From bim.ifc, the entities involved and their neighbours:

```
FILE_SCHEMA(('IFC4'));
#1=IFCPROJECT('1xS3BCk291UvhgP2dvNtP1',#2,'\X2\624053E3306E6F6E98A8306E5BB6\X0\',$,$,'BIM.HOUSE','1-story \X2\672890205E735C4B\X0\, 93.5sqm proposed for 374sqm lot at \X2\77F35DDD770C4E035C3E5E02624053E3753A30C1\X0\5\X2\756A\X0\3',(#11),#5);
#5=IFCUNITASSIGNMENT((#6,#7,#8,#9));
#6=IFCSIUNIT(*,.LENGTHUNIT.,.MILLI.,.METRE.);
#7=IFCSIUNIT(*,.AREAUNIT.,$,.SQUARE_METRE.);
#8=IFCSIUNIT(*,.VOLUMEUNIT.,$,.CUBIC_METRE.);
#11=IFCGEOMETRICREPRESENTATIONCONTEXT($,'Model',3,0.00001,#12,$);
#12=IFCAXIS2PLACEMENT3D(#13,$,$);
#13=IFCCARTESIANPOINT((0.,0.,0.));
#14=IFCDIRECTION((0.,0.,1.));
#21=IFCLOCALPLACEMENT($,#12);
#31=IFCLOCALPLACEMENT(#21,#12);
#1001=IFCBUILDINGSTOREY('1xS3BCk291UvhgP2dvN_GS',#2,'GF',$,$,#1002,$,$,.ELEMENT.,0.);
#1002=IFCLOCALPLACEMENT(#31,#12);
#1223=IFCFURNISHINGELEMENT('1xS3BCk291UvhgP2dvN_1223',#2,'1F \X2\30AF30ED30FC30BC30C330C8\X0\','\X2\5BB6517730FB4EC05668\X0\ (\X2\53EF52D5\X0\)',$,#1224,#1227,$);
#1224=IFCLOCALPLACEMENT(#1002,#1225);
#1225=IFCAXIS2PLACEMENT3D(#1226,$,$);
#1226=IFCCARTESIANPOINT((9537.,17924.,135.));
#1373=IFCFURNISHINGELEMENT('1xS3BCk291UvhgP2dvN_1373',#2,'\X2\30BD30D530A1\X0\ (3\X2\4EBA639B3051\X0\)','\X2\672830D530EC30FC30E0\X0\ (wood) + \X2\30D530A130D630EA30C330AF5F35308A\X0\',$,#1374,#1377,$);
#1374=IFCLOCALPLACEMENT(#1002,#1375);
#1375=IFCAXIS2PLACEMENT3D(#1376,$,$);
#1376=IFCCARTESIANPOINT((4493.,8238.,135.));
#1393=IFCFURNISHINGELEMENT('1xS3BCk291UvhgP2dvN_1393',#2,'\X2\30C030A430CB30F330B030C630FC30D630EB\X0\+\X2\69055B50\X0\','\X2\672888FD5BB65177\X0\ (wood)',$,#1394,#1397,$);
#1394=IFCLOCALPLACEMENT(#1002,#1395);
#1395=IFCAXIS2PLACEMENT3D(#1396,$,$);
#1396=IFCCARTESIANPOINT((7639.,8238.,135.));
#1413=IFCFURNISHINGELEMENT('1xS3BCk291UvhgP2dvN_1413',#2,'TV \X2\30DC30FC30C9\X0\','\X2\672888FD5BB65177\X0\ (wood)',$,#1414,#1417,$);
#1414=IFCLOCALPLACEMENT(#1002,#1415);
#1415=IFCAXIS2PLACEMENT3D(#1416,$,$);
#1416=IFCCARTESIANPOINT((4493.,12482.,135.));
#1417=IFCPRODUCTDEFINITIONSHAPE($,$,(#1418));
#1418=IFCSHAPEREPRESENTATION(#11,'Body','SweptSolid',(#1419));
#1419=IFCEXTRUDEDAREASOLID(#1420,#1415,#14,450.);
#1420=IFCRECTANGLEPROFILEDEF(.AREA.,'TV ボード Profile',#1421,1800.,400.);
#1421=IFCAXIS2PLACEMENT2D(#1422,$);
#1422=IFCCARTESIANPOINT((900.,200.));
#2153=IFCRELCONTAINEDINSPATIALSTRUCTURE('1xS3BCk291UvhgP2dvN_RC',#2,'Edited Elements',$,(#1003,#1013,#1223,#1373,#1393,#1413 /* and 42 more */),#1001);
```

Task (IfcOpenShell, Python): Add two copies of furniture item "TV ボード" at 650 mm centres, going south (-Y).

```python
import numpy as np
import ifcopenshell
import ifcopenshell.api.geometry
import ifcopenshell.api.root
import ifcopenshell.util.element
import ifcopenshell.util.placement

model = ifcopenshell.open("bim.ifc")


def reuse_history(source, copy):
    """copy_class also copies each property set's owner history, people and application; keep the originals."""
    for rel in copy.IsDefinedBy:
        if rel.is_a("IfcRelDefinesByProperties") and (history := rel.RelatingPropertyDefinition.OwnerHistory):
            rel.RelatingPropertyDefinition.OwnerHistory = source.OwnerHistory
            ifcopenshell.util.element.remove_deep2(model, history)


source = model.by_guid("1xS3BCk291UvhgP2dvN_1413")
base = ifcopenshell.util.placement.get_local_placement(source.ObjectPlacement)
step = np.array([0.0, -1.0, 0.0]) * 650.0

for i in range(1, 3):
    copy = ifcopenshell.api.root.copy_class(model, product=source)
    copy.Representation = ifcopenshell.util.element.copy_deep(
        model, source.Representation, exclude=["IfcGeometricRepresentationContext", "IfcRepresentationMap"]
    )
    reuse_history(source, copy)
    matrix = base.copy()
    matrix[:3, 3] += i * step
    print("added at", matrix[:3, 3].round(3) + 0.0)
    ifcopenshell.api.geometry.edit_object_placement(model, product=copy, matrix=matrix, is_si=False)

model.write("bim-out.ifc")
```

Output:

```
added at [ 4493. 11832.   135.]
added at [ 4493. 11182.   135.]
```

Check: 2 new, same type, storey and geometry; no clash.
